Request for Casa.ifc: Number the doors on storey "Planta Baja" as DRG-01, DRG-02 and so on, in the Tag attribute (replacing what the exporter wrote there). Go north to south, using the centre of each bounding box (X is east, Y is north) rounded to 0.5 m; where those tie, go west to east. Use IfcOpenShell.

First a look at what the model holds.

```python
import ifcopenshell
import ifcopenshell.util.element
import ifcopenshell.util.placement

model = ifcopenshell.open("Casa.ifc")
print(model.schema)
storey = next(s for s in model.by_type("IfcBuildingStorey") if s.Name == "Planta Baja")
doors = [e for e in ifcopenshell.util.element.get_decomposition(storey) if e.is_a("IfcDoor")]
for e in sorted(doors, key=lambda e: e.id()):
    origin = ifcopenshell.util.placement.get_local_placement(e.ObjectPlacement)[:3, 3]
    print(e.id(), e.Tag, e.Name, origin.round(2) + 0.0, sep=" | ")
```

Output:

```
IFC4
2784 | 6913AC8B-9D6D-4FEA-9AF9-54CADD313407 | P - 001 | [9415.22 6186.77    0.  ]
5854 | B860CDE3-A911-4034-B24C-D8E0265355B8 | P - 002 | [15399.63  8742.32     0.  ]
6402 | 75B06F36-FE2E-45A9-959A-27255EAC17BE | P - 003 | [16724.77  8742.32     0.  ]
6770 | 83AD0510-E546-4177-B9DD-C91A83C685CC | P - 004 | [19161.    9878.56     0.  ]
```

```python
import ifcopenshell
import ifcopenshell.geom
import ifcopenshell.util.element
import ifcopenshell.util.shape

model = ifcopenshell.open("Casa.ifc")
settings = ifcopenshell.geom.settings()
settings.set("use-world-coords", True)


def centre(element):
    shape = ifcopenshell.geom.create_shape(settings, element)
    return ifcopenshell.util.shape.get_bbox_centroid(shape.geometry)


storey = next(s for s in model.by_type("IfcBuildingStorey") if s.Name == "Planta Baja")
doors = [e for e in ifcopenshell.util.element.get_decomposition(storey) if e.is_a("IfcDoor")]

# Insertion points can sit at a corner or the storey origin, so sort by the geometry (in metres).
centres = {e: centre(e) for e in doors}
doors.sort(key=lambda e: (-round(centres[e][1] / 0.5), centres[e][0]))

for i, e in enumerate(doors, start=1):
    number = f"DRG-{i:02d}"
    e.Tag = number
    print(e.id(), number)

model.write("Casa_v2.ifc")
```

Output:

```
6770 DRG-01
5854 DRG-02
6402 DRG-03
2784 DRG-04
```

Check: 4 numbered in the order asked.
